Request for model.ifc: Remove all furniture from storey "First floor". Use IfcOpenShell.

First a look at what the model holds.

```python
import ifcopenshell
import ifcopenshell.util.element

model = ifcopenshell.open("model.ifc")
print(model.schema)
storey = next(s for s in model.by_type("IfcBuildingStorey") if s.Name == "First floor")
furniture = [e for e in ifcopenshell.util.element.get_decomposition(storey) if e.is_a("IfcFurnishingElement")]
seen = {}
for e in furniture:
    element_type = ifcopenshell.util.element.get_type(e)
    name = element_type.Name if element_type not in (None, e) else None
    seen[name] = seen.get(name, 0) + 1
for name, count in sorted(seen.items(), key=str):
    print(count, "x", name)
```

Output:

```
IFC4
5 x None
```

```python
import ifcopenshell
import ifcopenshell.api.root
import ifcopenshell.util.element

model = ifcopenshell.open("model.ifc")

storey = next(s for s in model.by_type("IfcBuildingStorey") if s.Name == "First floor")
furniture = [e for e in ifcopenshell.util.element.get_decomposition(storey) if e.is_a("IfcFurnishingElement")]

for e in furniture:
    ifcopenshell.api.root.remove_product(model, product=e)
print(len(furniture), "removed")

model.write("model-out.ifc")
```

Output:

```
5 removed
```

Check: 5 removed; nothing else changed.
